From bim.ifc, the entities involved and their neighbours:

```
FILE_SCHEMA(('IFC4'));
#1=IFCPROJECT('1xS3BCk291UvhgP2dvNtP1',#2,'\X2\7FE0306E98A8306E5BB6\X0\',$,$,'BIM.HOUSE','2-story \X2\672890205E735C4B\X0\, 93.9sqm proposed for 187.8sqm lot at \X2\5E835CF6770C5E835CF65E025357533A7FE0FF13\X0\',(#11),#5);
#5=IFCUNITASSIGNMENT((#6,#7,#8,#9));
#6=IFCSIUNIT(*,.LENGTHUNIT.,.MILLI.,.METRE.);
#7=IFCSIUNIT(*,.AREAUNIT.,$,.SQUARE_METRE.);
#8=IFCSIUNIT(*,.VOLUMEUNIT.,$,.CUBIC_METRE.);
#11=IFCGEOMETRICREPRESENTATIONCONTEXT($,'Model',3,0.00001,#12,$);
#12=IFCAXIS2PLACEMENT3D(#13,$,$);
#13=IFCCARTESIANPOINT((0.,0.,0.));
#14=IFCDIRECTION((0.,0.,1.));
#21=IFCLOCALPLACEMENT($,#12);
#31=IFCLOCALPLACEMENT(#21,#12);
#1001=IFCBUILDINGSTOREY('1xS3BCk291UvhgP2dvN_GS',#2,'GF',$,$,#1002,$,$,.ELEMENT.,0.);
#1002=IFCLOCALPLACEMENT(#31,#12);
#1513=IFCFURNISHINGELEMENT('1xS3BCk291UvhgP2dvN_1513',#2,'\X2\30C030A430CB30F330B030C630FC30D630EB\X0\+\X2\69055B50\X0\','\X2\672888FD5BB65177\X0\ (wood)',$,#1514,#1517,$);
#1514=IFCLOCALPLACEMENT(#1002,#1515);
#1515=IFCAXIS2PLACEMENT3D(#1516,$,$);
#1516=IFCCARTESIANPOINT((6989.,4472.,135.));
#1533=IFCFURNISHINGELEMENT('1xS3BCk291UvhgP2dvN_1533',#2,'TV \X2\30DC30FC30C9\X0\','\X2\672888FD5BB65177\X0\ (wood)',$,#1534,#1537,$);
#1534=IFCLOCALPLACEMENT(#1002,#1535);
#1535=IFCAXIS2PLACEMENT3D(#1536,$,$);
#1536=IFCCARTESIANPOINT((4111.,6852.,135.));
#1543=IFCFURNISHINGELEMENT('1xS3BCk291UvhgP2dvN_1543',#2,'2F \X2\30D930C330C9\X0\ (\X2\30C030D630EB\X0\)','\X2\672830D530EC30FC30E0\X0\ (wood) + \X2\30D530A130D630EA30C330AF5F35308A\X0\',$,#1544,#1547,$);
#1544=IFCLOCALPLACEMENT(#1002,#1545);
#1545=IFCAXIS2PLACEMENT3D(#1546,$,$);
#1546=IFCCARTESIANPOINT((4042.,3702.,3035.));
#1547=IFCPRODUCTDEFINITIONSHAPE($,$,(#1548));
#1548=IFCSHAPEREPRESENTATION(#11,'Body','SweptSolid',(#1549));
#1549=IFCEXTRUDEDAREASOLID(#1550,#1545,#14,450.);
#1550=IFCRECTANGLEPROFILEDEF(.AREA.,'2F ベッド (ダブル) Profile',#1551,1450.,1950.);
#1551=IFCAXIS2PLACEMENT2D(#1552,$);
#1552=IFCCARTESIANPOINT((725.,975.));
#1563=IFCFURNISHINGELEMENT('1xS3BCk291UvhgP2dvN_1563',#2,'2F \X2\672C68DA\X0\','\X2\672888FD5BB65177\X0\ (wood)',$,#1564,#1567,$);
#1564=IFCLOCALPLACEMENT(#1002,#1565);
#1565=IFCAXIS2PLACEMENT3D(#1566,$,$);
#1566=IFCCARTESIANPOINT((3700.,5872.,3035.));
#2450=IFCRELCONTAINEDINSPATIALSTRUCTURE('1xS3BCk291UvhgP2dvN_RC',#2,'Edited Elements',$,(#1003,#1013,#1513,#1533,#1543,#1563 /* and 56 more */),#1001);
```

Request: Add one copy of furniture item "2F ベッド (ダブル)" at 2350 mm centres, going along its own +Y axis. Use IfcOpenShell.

```python
import ifcopenshell
import ifcopenshell.api.geometry
import ifcopenshell.api.root
import ifcopenshell.util.element
import ifcopenshell.util.placement
import ifcopenshell.util.unit

model = ifcopenshell.open("bim.ifc")
unit_scale = ifcopenshell.util.unit.calculate_unit_scale(model)


def reuse_history(source, copy):
    """copy_class also copies each property set's owner history, people and application; keep the originals."""
    for rel in copy.IsDefinedBy:
        if rel.is_a("IfcRelDefinesByProperties") and (history := rel.RelatingPropertyDefinition.OwnerHistory):
            rel.RelatingPropertyDefinition.OwnerHistory = source.OwnerHistory
            ifcopenshell.util.element.remove_deep2(model, history)


source = model.by_guid("1xS3BCk291UvhgP2dvN_1543")
base = ifcopenshell.util.placement.get_local_placement(source.ObjectPlacement)
step = base[:3, 1] * 2.35 / unit_scale

for i in range(1, 2):
    copy = ifcopenshell.api.root.copy_class(model, product=source)
    copy.Representation = ifcopenshell.util.element.copy_deep(
        model, source.Representation, exclude=["IfcGeometricRepresentationContext", "IfcRepresentationMap"]
    )
    reuse_history(source, copy)
    matrix = base.copy()
    matrix[:3, 3] += i * step
    print("added at", matrix[:3, 3].round(3) + 0.0)
    ifcopenshell.api.geometry.edit_object_placement(model, product=copy, matrix=matrix, is_si=False)

model.write("bim_rev.ifc")
```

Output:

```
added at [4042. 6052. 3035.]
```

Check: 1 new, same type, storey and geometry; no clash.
